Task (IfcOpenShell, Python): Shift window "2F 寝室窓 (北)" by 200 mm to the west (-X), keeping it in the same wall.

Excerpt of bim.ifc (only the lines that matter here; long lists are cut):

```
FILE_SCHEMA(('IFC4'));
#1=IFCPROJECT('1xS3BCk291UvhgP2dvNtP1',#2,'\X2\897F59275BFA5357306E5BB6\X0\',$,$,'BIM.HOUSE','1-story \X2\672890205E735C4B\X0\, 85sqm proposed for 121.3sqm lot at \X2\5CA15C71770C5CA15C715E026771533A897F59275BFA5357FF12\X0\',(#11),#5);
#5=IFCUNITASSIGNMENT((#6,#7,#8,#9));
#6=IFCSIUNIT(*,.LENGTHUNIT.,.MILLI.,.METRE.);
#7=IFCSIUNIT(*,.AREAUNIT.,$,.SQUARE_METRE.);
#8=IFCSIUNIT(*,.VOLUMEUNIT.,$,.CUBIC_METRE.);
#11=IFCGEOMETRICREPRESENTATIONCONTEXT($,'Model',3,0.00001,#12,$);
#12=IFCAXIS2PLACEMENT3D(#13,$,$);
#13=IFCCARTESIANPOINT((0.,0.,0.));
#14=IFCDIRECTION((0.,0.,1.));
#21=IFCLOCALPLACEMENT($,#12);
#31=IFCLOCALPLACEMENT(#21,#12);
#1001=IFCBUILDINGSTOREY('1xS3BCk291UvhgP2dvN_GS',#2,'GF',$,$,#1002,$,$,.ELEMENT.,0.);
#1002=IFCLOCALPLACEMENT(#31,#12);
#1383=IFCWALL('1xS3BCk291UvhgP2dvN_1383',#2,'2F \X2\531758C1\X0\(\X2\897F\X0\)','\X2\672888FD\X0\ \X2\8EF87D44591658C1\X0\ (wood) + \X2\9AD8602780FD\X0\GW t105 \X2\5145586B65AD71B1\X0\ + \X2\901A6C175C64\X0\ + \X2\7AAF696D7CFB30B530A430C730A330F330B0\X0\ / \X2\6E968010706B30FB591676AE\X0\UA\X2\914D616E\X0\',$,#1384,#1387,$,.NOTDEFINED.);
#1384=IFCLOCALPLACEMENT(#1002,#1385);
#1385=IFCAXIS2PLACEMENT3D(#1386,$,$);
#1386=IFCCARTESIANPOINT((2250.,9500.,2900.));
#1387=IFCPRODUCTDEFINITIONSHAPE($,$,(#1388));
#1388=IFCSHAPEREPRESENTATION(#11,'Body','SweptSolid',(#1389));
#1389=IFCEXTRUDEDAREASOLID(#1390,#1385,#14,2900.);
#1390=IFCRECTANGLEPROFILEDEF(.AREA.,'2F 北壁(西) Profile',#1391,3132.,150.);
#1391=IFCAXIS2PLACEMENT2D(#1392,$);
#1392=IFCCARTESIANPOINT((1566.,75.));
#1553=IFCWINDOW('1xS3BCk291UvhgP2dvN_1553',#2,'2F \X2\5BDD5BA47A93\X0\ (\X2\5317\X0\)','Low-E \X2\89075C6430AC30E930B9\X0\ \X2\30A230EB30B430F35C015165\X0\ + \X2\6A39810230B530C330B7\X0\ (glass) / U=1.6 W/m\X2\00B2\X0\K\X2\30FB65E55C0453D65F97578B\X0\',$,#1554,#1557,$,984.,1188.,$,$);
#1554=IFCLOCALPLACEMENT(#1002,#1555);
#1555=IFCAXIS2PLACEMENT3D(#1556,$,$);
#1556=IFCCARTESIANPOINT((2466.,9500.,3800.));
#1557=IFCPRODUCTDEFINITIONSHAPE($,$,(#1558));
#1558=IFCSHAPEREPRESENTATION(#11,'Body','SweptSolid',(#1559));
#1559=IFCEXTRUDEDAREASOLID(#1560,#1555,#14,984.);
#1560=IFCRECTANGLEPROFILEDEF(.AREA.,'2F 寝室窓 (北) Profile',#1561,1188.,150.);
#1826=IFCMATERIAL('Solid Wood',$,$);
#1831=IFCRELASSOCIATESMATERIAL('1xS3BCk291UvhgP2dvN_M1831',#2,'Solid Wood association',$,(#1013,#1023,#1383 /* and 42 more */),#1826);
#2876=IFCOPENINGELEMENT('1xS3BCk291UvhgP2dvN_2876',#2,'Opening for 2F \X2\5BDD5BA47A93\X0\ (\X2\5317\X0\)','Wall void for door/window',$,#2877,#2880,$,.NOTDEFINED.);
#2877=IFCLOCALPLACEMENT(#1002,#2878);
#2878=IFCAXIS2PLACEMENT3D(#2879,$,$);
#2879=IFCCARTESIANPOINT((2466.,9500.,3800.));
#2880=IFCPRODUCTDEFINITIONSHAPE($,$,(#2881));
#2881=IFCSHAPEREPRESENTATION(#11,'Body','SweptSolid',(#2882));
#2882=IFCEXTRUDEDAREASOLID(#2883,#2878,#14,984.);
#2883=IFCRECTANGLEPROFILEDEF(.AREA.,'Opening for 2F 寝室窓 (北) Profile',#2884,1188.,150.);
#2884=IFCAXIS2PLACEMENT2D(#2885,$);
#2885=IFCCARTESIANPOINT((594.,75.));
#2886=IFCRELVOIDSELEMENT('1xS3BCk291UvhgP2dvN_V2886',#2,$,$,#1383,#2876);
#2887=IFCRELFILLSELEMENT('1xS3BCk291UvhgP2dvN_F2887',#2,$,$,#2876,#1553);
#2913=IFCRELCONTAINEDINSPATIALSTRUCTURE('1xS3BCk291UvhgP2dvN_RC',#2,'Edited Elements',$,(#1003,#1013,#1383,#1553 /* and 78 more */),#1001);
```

```python
import ifcopenshell
import ifcopenshell.api.geometry
import ifcopenshell.util.placement
import ifcopenshell.util.unit

model = ifcopenshell.open("bim.ifc")
unit_scale = ifcopenshell.util.unit.calculate_unit_scale(model)

window = model.by_id(1553)
opening = window.FillsVoids[0].RelatingOpeningElement
wall = opening.VoidsElements[0].RelatingBuildingElement

wall_matrix = ifcopenshell.util.placement.get_local_placement(wall.ObjectPlacement)
shift = wall_matrix[:3, 0] * -0.2 / unit_scale
before = ifcopenshell.util.placement.get_local_placement(window.ObjectPlacement)[:3, 3].copy()

# The window is not placed relative to its opening, so move both.
for product in (opening, window):
    matrix = ifcopenshell.util.placement.get_local_placement(product.ObjectPlacement)
    matrix[:3, 3] += shift
    ifcopenshell.api.geometry.edit_object_placement(model, product=product, matrix=matrix, is_si=False)

after = ifcopenshell.util.placement.get_local_placement(window.ObjectPlacement)[:3, 3]
print("window moved by", (after - before).round(3) + 0.0)

model.write("bim_rev.ifc")
```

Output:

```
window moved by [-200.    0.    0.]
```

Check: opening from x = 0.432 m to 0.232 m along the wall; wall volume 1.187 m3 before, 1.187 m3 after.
